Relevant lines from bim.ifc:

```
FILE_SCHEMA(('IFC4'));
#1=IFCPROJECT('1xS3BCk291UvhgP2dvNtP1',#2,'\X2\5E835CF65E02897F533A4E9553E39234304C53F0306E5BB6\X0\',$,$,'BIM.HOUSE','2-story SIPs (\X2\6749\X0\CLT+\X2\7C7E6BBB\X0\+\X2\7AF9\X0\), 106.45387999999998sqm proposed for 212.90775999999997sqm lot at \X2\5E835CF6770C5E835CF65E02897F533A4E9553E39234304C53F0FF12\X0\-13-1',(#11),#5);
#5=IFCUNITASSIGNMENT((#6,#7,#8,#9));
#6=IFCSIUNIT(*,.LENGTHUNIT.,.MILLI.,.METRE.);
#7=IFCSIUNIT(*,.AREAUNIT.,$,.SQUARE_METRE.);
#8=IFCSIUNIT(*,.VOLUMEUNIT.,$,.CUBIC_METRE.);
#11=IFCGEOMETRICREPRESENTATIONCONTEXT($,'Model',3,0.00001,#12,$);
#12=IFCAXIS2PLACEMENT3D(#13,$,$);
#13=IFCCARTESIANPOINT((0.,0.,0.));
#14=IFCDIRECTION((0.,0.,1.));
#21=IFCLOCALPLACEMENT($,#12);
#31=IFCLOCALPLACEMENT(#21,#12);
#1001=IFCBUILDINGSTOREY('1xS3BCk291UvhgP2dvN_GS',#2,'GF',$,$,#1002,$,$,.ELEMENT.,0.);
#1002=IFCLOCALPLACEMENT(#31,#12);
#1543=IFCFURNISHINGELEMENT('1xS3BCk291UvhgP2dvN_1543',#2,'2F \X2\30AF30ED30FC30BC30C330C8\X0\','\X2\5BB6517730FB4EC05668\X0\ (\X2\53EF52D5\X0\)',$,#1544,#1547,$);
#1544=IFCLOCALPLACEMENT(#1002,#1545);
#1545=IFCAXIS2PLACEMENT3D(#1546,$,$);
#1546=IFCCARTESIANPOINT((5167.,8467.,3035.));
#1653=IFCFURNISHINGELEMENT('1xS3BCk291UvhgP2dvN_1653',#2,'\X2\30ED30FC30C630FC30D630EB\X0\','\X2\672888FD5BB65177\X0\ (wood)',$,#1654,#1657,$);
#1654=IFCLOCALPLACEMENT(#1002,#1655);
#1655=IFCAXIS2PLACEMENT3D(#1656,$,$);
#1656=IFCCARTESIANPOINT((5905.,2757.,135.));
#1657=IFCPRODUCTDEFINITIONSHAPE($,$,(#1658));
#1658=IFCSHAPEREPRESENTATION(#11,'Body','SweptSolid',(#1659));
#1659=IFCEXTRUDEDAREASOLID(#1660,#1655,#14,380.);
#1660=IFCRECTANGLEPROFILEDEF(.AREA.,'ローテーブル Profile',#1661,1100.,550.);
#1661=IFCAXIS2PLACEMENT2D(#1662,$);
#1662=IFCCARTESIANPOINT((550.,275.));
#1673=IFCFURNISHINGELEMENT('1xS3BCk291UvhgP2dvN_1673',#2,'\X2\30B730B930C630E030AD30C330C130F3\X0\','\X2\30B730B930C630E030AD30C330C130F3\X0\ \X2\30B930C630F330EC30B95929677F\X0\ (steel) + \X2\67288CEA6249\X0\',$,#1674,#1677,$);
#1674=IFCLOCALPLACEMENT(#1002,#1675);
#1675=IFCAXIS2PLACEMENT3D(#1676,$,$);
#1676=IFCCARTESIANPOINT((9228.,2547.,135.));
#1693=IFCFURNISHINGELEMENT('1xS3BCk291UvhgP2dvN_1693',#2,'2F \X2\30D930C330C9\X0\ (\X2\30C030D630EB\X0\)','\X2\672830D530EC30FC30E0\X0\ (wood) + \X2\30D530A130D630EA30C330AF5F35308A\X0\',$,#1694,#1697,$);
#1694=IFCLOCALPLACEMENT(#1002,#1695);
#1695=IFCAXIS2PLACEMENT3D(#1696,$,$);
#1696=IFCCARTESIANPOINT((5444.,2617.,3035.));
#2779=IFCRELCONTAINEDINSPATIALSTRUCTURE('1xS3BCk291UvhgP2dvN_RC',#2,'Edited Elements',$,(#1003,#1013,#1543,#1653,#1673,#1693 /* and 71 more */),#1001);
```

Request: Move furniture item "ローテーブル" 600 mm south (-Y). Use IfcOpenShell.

```python
import ifcopenshell
import ifcopenshell.api.geometry
import ifcopenshell.util.placement
import ifcopenshell.util.unit

model = ifcopenshell.open("bim.ifc")
unit_scale = ifcopenshell.util.unit.calculate_unit_scale(model)

item = model.by_guid("1xS3BCk291UvhgP2dvN_1653")
matrix = ifcopenshell.util.placement.get_local_placement(item.ObjectPlacement)
matrix[1, 3] -= 0.6 / unit_scale
ifcopenshell.api.geometry.edit_object_placement(model, product=item, matrix=matrix, is_si=False)

print(ifcopenshell.util.placement.get_local_placement(item.ObjectPlacement).round(3) + 0.0)

model.write("bim_rev.ifc")
```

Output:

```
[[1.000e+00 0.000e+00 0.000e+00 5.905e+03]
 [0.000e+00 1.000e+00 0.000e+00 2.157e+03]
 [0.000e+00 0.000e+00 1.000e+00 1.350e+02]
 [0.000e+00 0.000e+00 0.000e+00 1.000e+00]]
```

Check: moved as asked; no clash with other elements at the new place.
